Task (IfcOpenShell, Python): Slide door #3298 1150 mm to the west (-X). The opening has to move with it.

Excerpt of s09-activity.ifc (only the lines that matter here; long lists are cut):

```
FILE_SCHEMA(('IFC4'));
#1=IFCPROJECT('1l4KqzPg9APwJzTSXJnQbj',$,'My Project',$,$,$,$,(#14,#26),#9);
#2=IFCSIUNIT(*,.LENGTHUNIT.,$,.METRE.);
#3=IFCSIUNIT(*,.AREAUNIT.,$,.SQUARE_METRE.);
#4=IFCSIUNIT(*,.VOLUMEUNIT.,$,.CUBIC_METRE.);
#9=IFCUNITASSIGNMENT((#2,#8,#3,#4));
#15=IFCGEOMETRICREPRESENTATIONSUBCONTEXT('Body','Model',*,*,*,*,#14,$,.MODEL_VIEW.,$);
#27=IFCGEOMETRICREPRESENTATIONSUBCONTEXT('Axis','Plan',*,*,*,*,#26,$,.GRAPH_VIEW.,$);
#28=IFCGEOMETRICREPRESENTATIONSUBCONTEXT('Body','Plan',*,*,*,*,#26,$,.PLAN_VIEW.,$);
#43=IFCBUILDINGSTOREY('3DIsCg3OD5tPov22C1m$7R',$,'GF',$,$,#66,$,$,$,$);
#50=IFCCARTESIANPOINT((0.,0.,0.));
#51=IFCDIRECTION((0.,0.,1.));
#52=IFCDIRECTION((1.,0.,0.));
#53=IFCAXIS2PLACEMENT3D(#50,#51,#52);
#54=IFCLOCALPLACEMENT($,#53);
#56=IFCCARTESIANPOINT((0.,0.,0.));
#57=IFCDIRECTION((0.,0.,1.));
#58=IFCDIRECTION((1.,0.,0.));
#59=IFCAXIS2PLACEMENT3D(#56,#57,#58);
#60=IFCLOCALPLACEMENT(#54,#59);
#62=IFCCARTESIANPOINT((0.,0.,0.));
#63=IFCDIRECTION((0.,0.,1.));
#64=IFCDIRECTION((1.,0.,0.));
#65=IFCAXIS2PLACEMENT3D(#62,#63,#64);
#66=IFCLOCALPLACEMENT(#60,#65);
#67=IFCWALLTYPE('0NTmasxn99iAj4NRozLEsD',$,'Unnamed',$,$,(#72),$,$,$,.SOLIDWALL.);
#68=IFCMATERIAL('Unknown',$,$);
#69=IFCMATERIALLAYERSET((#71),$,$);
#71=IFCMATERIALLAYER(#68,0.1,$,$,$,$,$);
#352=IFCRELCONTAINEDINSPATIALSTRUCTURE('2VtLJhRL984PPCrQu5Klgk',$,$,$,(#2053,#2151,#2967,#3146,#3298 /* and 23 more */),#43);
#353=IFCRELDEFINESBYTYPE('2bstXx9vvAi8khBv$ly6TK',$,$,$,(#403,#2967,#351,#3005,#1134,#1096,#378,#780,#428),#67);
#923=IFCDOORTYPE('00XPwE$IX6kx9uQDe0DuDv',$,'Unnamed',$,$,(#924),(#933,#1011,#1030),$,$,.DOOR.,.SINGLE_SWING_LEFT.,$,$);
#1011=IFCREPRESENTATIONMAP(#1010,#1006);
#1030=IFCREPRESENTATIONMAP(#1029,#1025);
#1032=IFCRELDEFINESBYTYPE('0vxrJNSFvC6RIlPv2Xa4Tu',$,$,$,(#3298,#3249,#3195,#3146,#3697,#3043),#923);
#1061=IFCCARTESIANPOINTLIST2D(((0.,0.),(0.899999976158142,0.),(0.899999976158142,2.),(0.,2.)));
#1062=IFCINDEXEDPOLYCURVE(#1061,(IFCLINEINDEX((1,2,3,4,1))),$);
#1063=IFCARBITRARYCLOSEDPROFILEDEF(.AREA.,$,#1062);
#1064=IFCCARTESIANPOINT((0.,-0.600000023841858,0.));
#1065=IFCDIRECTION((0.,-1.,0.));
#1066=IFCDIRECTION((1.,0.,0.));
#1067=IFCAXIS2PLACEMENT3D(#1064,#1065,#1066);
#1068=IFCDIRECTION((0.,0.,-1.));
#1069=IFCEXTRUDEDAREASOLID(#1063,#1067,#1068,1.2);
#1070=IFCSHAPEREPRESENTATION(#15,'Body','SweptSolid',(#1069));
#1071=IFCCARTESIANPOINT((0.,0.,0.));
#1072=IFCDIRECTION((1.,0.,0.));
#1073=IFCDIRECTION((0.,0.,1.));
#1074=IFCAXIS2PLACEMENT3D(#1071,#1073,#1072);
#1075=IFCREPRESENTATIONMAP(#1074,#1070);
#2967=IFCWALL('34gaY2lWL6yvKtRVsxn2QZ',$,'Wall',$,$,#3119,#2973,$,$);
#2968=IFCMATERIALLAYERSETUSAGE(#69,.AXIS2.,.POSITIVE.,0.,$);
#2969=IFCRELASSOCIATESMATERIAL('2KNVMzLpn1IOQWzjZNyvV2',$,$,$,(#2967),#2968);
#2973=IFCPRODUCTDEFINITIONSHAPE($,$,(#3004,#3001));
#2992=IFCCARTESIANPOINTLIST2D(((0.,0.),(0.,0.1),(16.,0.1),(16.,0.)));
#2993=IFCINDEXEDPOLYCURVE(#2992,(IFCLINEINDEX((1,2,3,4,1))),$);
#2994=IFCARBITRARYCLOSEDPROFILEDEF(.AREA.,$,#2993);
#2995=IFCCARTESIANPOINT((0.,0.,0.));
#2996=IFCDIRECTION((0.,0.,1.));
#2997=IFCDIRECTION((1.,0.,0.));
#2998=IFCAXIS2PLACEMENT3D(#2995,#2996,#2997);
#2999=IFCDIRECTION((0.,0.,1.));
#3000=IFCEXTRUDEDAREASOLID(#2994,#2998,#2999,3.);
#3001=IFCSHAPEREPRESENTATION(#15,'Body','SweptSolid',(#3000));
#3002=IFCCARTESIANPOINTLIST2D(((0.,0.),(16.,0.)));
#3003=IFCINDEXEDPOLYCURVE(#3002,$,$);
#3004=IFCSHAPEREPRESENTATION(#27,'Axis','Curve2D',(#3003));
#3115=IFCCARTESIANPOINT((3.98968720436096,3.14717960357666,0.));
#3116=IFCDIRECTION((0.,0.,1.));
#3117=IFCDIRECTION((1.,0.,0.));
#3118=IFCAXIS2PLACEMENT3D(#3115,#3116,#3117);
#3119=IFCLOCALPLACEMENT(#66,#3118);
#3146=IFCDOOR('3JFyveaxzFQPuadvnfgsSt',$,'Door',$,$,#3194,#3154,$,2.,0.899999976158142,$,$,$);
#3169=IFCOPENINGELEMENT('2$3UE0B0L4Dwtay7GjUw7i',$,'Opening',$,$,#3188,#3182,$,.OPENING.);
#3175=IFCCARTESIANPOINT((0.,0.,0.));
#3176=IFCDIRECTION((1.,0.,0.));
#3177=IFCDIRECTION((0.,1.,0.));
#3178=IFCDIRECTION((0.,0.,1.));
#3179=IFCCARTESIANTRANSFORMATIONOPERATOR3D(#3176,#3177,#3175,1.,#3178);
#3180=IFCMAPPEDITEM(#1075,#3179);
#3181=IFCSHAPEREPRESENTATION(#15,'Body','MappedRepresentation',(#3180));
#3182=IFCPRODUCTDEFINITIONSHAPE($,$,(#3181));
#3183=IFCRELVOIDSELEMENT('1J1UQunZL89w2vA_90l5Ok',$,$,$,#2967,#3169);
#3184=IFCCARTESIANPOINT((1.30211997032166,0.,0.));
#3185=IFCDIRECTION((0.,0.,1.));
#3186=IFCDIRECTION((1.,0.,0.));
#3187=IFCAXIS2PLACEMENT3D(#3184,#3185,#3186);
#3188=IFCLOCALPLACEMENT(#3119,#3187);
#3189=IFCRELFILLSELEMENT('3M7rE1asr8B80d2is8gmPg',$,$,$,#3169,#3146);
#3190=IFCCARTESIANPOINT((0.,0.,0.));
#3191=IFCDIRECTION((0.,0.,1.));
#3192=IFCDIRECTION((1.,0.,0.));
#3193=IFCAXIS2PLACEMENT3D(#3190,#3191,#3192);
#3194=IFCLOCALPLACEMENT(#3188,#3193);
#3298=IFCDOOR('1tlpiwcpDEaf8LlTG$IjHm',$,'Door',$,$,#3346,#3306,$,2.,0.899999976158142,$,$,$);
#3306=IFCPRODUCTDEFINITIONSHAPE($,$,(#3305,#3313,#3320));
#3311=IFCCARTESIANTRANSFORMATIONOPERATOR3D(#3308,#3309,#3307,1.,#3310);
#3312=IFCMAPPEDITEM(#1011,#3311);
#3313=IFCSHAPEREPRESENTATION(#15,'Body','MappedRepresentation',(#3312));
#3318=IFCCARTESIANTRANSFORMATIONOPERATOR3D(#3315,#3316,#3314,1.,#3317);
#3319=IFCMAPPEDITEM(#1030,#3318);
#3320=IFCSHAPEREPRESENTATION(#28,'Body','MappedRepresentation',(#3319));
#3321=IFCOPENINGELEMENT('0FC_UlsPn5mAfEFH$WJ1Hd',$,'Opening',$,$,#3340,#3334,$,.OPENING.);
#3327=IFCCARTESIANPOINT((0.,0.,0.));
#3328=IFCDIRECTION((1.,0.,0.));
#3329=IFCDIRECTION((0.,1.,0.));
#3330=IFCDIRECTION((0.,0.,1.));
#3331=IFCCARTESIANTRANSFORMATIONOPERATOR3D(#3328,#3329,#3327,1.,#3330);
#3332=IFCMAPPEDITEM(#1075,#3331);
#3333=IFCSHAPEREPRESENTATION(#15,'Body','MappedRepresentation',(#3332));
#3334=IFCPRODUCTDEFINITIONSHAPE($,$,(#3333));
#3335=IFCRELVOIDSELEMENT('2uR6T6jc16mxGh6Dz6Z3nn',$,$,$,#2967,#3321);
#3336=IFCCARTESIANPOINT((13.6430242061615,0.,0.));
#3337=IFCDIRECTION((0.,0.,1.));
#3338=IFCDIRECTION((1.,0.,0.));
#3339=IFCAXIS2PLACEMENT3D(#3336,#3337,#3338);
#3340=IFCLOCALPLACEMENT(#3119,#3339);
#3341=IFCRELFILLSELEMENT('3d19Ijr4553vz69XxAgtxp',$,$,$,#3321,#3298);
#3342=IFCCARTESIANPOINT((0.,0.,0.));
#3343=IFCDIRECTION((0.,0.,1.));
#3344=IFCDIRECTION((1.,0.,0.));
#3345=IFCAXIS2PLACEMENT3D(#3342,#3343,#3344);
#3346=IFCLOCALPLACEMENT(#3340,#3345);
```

```python
import ifcopenshell
import ifcopenshell.api.geometry
import ifcopenshell.util.placement
import ifcopenshell.util.unit

model = ifcopenshell.open("s09-activity.ifc")
unit_scale = ifcopenshell.util.unit.calculate_unit_scale(model)

door = model.by_guid("1tlpiwcpDEaf8LlTG$IjHm")
opening = door.FillsVoids[0].RelatingOpeningElement
wall = opening.VoidsElements[0].RelatingBuildingElement

wall_matrix = ifcopenshell.util.placement.get_local_placement(wall.ObjectPlacement)
shift = wall_matrix[:3, 0] * -1.15 / unit_scale
before = ifcopenshell.util.placement.get_local_placement(door.ObjectPlacement)[:3, 3].copy()

# The door is placed relative to its opening, so it follows when the opening moves.
matrix = ifcopenshell.util.placement.get_local_placement(opening.ObjectPlacement)
matrix[:3, 3] += shift
ifcopenshell.api.geometry.edit_object_placement(
    model, product=opening, matrix=matrix, is_si=False, should_transform_children=True
)

after = ifcopenshell.util.placement.get_local_placement(door.ObjectPlacement)[:3, 3]
print("door moved by", (after - before).round(3) + 0.0)

model.write("s09-activity_edited.ifc")
```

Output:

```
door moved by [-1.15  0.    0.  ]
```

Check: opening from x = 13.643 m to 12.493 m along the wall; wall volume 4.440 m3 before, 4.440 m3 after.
